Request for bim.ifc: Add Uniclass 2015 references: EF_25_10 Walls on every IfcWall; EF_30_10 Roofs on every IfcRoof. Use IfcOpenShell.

First a look at what the model holds.

```python
import ifcopenshell

model = ifcopenshell.open("bim.ifc")
print(model.schema)
print("classifications:", [c.Name for c in model.by_type("IfcClassification")])
for ifc_class in ("IfcDoor", "IfcRoof", "IfcStair", "IfcWall", "IfcWindow"):
    print(ifc_class, len(model.by_type(ifc_class)))
```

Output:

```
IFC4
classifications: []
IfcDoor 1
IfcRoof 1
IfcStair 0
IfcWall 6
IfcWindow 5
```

```python
import ifcopenshell
import ifcopenshell.api.classification

model = ifcopenshell.open("bim.ifc")

system = ifcopenshell.api.classification.add_classification(model, classification="Uniclass 2015")

codes = {
    "IfcWall": ("EF_25_10", "Walls"),
    "IfcRoof": ("EF_30_10", "Roofs"),
}
for ifc_class, (code, name) in codes.items():
    products = model.by_type(ifc_class)
    ifcopenshell.api.classification.add_reference(
        model, products=products, classification=system, identification=code, name=name
    )
    print(code, len(products))

model.write("bim_edited.ifc")
```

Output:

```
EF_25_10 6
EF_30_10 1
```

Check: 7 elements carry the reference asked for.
